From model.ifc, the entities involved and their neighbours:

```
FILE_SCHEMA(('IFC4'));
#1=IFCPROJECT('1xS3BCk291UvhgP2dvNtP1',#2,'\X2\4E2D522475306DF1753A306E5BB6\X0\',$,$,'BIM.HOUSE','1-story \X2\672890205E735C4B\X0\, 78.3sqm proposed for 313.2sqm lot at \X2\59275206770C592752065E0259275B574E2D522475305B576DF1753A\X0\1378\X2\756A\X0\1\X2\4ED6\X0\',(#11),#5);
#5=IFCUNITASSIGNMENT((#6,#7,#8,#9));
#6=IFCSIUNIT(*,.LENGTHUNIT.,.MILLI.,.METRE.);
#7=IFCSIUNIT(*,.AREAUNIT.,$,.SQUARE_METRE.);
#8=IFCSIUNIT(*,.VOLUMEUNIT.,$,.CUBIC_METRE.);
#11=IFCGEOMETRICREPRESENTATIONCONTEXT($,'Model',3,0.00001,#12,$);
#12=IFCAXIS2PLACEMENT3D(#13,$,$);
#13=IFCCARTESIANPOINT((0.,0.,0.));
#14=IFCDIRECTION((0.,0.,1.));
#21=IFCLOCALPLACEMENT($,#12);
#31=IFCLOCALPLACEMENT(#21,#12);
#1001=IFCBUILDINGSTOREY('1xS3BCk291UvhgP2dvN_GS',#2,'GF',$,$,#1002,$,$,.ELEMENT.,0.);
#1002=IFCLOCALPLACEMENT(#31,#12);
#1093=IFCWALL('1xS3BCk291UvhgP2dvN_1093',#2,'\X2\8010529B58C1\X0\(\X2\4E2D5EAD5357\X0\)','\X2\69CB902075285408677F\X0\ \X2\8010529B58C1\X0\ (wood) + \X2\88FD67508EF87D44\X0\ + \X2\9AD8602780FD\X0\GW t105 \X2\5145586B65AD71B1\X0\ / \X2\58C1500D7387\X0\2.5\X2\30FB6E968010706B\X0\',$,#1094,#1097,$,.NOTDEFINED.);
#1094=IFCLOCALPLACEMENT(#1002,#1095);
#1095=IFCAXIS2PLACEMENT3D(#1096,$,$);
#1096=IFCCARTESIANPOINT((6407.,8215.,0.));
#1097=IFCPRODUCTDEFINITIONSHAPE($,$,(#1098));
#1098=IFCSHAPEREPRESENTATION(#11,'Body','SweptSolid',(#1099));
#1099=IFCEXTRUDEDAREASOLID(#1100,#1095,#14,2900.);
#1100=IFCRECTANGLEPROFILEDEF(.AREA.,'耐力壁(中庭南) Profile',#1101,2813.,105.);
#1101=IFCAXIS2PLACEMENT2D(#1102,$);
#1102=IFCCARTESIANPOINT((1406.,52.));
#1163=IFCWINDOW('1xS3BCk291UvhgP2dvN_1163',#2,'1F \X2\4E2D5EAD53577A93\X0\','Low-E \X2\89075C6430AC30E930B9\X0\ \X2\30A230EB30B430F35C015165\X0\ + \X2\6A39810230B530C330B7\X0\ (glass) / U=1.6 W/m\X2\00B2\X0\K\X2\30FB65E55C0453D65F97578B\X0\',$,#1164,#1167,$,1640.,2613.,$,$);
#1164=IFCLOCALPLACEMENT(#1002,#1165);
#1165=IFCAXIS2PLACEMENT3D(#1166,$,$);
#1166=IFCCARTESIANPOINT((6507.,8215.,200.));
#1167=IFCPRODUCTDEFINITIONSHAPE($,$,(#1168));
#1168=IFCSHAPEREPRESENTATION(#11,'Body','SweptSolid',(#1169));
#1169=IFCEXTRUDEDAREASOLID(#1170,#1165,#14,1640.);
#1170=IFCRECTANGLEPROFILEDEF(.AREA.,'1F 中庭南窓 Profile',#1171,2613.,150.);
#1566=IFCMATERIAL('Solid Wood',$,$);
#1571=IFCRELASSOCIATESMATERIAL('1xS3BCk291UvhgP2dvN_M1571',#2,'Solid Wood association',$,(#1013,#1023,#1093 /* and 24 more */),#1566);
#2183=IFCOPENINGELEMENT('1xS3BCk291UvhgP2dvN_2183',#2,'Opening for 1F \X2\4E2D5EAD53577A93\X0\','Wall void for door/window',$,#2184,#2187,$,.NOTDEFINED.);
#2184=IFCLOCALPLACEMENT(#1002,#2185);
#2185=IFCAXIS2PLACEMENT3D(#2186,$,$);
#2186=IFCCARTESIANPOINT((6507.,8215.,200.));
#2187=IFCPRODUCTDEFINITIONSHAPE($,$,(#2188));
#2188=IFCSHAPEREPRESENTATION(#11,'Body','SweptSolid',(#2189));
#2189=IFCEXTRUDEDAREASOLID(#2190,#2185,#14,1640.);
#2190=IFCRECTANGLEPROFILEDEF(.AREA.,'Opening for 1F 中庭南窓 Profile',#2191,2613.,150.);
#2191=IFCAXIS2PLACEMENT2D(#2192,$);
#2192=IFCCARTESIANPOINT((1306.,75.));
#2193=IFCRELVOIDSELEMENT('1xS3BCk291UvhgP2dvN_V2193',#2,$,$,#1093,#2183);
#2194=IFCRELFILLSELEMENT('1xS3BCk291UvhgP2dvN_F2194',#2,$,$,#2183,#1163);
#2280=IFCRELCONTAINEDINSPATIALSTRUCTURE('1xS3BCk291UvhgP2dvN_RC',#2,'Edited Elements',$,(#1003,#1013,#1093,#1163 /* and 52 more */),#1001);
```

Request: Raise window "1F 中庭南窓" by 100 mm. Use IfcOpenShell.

```python
import numpy as np
import ifcopenshell
import ifcopenshell.api.geometry
import ifcopenshell.util.placement
import ifcopenshell.util.unit

model = ifcopenshell.open("model.ifc")
unit_scale = ifcopenshell.util.unit.calculate_unit_scale(model)

window = model.by_guid("1xS3BCk291UvhgP2dvN_1163")
opening = window.FillsVoids[0].RelatingOpeningElement
dz = 100.0

shift = np.array([0.0, 0.0, dz])
# The window is not placed relative to its opening, so move both.
for product in (opening, window):
    matrix = ifcopenshell.util.placement.get_local_placement(product.ObjectPlacement)
    matrix[:3, 3] += shift
    ifcopenshell.api.geometry.edit_object_placement(model, product=product, matrix=matrix, is_si=False)

print(f"moved by {dz * unit_scale:+.3f} m")

model.write("model_updated.ifc")
```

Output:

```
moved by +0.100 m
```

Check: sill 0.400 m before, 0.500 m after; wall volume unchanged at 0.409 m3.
